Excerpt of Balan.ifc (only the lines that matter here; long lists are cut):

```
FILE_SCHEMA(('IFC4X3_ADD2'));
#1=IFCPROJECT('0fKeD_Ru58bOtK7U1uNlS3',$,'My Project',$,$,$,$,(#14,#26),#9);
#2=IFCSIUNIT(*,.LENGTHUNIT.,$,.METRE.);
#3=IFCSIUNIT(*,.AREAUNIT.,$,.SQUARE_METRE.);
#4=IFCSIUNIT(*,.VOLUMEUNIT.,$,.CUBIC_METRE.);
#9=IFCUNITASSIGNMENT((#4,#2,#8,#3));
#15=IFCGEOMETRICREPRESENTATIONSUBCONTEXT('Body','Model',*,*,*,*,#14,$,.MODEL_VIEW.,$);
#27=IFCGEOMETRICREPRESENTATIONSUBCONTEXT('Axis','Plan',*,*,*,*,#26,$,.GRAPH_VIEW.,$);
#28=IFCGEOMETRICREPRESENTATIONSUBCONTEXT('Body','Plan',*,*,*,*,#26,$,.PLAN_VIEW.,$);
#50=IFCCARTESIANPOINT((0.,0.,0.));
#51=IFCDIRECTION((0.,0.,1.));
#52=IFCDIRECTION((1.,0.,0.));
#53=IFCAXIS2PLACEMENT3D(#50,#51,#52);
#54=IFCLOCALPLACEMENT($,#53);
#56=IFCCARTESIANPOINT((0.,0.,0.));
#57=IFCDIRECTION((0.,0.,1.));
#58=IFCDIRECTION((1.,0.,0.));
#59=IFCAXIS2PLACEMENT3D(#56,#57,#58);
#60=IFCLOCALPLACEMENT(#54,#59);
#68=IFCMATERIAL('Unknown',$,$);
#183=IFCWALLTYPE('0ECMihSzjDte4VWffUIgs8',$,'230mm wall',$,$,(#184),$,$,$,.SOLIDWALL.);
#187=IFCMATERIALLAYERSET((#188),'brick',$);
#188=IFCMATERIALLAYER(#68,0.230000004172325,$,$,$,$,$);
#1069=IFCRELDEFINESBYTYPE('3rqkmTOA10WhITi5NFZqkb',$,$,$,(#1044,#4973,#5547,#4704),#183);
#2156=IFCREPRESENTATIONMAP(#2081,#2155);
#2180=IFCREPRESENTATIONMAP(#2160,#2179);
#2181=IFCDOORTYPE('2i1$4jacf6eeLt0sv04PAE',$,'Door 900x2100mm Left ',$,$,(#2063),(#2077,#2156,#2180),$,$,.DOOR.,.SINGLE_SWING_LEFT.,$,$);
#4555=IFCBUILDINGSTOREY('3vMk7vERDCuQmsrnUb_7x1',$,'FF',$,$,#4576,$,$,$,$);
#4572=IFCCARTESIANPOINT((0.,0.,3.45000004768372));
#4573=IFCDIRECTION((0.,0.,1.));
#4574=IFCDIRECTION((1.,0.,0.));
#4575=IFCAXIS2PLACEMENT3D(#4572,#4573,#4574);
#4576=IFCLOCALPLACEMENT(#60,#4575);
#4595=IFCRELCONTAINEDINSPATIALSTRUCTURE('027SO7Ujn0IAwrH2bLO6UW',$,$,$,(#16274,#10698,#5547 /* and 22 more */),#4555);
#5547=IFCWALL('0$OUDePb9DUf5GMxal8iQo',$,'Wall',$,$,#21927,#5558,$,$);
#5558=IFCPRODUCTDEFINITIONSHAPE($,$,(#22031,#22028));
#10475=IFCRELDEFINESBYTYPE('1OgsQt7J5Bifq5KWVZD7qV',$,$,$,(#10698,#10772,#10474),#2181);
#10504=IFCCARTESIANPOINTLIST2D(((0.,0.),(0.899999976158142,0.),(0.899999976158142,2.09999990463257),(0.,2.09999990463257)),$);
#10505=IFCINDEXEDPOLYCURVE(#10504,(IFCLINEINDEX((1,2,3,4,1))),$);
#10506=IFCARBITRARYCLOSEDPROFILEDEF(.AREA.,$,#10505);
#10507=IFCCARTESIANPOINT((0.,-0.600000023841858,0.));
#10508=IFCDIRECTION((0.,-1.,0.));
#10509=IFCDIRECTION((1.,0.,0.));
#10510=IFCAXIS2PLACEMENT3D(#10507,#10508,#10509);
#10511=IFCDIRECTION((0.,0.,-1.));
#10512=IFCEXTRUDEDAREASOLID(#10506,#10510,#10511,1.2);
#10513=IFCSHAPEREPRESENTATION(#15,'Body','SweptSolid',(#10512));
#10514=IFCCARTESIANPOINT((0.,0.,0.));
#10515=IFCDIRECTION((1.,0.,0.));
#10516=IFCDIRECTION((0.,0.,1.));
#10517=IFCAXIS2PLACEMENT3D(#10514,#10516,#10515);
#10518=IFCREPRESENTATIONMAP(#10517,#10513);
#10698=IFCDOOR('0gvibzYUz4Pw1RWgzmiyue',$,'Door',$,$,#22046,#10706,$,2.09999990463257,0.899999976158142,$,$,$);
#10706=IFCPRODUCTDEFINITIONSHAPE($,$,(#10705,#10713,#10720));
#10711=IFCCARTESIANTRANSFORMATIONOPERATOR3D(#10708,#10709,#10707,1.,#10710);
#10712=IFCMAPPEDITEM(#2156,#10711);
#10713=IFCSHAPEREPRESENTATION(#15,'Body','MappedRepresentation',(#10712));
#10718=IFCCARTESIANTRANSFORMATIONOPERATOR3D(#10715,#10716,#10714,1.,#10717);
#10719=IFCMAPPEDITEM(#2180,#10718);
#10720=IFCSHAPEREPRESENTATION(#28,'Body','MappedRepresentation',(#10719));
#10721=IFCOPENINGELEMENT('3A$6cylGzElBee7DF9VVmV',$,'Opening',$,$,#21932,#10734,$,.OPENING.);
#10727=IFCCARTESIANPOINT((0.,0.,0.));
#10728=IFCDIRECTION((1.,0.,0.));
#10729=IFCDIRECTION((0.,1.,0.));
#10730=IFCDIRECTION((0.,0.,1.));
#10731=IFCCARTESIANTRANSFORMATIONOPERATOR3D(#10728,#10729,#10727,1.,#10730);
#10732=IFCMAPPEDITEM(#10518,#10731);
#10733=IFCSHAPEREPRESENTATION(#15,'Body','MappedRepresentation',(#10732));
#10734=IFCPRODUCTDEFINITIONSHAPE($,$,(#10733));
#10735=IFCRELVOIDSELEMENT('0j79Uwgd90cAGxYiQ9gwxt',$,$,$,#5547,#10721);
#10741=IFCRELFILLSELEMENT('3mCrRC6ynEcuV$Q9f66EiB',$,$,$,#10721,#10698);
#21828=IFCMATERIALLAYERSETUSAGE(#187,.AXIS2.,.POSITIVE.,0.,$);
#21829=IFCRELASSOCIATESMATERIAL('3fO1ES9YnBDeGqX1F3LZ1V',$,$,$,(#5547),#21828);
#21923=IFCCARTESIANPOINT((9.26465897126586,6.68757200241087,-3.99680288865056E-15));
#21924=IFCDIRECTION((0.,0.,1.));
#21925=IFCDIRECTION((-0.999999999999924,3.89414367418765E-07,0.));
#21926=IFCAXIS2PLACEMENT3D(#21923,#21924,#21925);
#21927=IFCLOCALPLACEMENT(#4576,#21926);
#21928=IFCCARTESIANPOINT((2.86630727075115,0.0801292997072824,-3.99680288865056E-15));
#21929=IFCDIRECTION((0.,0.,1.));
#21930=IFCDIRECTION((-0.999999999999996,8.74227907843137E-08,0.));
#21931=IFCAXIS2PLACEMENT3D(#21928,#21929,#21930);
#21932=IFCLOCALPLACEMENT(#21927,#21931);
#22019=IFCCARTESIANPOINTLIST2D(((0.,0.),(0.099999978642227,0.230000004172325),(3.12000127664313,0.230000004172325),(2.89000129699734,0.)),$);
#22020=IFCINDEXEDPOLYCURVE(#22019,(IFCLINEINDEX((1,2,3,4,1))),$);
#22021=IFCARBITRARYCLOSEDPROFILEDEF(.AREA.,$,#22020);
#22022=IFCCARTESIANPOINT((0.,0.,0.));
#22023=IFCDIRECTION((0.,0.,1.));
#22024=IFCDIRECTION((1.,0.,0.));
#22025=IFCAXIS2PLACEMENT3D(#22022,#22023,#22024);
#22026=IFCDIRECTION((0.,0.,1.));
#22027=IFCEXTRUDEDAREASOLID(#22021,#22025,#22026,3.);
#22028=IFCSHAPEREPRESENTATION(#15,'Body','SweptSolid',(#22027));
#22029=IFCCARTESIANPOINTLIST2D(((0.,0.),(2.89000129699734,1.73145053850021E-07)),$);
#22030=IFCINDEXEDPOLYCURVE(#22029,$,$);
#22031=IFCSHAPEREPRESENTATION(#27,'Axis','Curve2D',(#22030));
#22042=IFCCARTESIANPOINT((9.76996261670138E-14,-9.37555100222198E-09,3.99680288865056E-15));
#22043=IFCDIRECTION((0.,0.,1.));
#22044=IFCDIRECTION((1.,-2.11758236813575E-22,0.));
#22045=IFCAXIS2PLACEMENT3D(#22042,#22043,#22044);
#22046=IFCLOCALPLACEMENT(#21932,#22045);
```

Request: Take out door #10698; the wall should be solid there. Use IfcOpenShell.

```python
import ifcopenshell
import ifcopenshell.api.feature
import ifcopenshell.api.root
import ifcopenshell.geom
import ifcopenshell.util.shape

model = ifcopenshell.open("Balan.ifc")
settings = ifcopenshell.geom.settings()


def volume(element):
    """Net volume in cubic metres, openings subtracted."""
    shape = ifcopenshell.geom.create_shape(settings, element)
    return ifcopenshell.util.shape.get_volume(shape.geometry)


door = model.by_guid("0gvibzYUz4Pw1RWgzmiyue")
opening = door.FillsVoids[0].RelatingOpeningElement
wall = opening.VoidsElements[0].RelatingBuildingElement
before = volume(wall)

ifcopenshell.api.root.remove_product(model, product=door)
ifcopenshell.api.feature.remove_feature(model, feature=opening)

after = volume(wall)

print(f"wall volume {before:.3f} -> {after:.3f} m3")

model.write("Balan_rev.ifc")
```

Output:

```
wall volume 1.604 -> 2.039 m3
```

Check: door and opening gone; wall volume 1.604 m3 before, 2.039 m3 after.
